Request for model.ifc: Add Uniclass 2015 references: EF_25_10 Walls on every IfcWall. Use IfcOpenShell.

First a look at what the model holds.

```python
import ifcopenshell

model = ifcopenshell.open("model.ifc")
print(model.schema)
print("classifications:", [c.Name for c in model.by_type("IfcClassification")])
for ifc_class in ("IfcDoor", "IfcRoof", "IfcStair", "IfcWall", "IfcWindow"):
    print(ifc_class, len(model.by_type(ifc_class)))
```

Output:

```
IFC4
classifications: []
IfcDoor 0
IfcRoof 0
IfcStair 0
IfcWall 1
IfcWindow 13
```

```python
import ifcopenshell
import ifcopenshell.api.classification

model = ifcopenshell.open("model.ifc")

system = ifcopenshell.api.classification.add_classification(model, classification="Uniclass 2015")

codes = {
    "IfcWall": ("EF_25_10", "Walls"),
}
for ifc_class, (code, name) in codes.items():
    products = model.by_type(ifc_class)
    ifcopenshell.api.classification.add_reference(
        model, products=products, classification=system, identification=code, name=name
    )
    print(code, len(products))

model.write("model_updated.ifc")
```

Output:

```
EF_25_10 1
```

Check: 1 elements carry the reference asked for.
